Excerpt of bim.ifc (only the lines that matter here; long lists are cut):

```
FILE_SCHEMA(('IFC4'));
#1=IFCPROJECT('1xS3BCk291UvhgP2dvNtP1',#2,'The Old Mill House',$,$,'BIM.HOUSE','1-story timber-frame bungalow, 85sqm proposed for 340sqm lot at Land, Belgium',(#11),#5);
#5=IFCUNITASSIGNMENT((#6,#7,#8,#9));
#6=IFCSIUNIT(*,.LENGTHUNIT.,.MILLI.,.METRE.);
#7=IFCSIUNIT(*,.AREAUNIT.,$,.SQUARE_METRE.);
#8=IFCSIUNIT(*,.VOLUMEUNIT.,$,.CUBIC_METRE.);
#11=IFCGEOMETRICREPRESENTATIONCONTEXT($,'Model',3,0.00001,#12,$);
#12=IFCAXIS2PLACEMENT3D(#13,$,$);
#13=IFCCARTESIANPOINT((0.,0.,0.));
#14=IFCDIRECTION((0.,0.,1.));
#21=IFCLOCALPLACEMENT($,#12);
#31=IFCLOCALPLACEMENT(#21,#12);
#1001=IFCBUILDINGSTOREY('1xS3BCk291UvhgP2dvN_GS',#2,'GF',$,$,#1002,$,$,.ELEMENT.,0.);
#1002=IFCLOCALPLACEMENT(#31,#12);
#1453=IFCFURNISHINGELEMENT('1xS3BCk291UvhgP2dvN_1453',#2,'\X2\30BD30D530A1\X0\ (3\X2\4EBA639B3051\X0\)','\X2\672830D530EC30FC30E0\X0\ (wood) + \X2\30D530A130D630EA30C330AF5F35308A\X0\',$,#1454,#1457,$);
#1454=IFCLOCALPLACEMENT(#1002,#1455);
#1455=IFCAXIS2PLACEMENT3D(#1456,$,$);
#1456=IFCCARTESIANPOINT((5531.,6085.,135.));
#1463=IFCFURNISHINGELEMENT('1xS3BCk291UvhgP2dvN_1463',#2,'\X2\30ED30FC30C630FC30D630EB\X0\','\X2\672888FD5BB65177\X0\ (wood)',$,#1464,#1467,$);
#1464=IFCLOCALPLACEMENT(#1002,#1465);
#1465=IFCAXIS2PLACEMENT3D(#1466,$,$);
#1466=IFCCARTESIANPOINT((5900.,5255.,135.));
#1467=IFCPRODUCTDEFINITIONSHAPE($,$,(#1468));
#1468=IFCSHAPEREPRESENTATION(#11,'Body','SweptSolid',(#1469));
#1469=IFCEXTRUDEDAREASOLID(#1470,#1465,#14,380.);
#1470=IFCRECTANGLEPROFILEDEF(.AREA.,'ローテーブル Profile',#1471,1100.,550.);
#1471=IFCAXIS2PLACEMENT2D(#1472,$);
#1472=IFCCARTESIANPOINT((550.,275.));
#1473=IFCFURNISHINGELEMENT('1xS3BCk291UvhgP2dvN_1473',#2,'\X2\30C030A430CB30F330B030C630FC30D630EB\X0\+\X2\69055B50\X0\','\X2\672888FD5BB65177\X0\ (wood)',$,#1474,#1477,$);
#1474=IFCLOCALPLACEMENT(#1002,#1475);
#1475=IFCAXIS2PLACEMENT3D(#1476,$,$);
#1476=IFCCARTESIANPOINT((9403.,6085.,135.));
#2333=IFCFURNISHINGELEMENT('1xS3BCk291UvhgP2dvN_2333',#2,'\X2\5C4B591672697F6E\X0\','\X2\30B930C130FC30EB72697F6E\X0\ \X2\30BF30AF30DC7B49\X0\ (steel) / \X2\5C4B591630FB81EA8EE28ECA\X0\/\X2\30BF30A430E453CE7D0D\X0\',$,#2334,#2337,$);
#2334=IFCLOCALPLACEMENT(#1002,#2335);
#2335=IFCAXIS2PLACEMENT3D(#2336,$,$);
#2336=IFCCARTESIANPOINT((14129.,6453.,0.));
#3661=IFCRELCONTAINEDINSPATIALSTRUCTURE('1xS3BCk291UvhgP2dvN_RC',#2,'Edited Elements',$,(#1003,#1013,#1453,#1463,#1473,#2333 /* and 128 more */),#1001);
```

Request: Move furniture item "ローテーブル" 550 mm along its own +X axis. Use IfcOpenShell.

```python
import ifcopenshell
import ifcopenshell.api.geometry
import ifcopenshell.util.placement

model = ifcopenshell.open("bim.ifc")

item = model.by_guid("1xS3BCk291UvhgP2dvN_1463")
matrix = ifcopenshell.util.placement.get_local_placement(item.ObjectPlacement)
matrix[:3, 3] += matrix[:3, 0] * 550.0
ifcopenshell.api.geometry.edit_object_placement(model, product=item, matrix=matrix, is_si=False)

print(ifcopenshell.util.placement.get_local_placement(item.ObjectPlacement).round(3) + 0.0)

model.write("bim_updated.ifc")
```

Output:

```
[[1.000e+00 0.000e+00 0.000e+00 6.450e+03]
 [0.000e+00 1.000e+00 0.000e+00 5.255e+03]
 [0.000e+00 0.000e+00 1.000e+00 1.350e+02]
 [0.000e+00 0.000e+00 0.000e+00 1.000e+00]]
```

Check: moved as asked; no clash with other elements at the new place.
